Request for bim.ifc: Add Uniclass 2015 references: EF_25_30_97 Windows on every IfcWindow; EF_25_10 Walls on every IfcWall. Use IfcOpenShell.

First a look at what the model holds.

```python
import ifcopenshell

model = ifcopenshell.open("bim.ifc")
print(model.schema)
print("classifications:", [c.Name for c in model.by_type("IfcClassification")])
for ifc_class in ("IfcDoor", "IfcRoof", "IfcStair", "IfcWall", "IfcWindow"):
    print(ifc_class, len(model.by_type(ifc_class)))
```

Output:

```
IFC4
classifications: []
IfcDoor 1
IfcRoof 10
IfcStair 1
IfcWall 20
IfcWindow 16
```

```python
import ifcopenshell
import ifcopenshell.api.classification

model = ifcopenshell.open("bim.ifc")

system = ifcopenshell.api.classification.add_classification(model, classification="Uniclass 2015")

codes = {
    "IfcWindow": ("EF_25_30_97", "Windows"),
    "IfcWall": ("EF_25_10", "Walls"),
}
for ifc_class, (code, name) in codes.items():
    products = model.by_type(ifc_class)
    ifcopenshell.api.classification.add_reference(
        model, products=products, classification=system, identification=code, name=name
    )
    print(code, len(products))

model.write("bim_updated.ifc")
```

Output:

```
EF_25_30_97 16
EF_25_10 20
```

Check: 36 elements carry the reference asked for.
